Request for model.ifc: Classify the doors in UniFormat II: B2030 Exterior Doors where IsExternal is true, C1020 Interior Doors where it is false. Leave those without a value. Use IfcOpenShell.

First a look at what the model holds.

```python
import ifcopenshell
import ifcopenshell.util.element

model = ifcopenshell.open("model.ifc")
print(model.schema)
print("classifications:", [c.Name for c in model.by_type("IfcClassification")])
values = [ifcopenshell.util.element.get_pset(e, "Pset_DoorCommon", "IsExternal") for e in model.by_type("IfcDoor")]
for value in (True, False, None):
    print("IsExternal", value, values.count(value))
```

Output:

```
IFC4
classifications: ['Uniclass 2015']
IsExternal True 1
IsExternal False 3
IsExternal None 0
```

```python
import ifcopenshell
import ifcopenshell.api.classification
import ifcopenshell.util.element

model = ifcopenshell.open("model.ifc")

system = ifcopenshell.api.classification.add_classification(model, classification="UniFormat II")

doors = model.by_type("IfcDoor")
external = {e: ifcopenshell.util.element.get_pset(e, "Pset_DoorCommon", "IsExternal") for e in doors}
for flag, code, name in ((True, "B2030", "Exterior Doors"), (False, "C1020", "Interior Doors")):
    products = [e for e in doors if external[e] is flag]
    ifcopenshell.api.classification.add_reference(
        model, products=products, classification=system, identification=code, name=name
    )
    print(code, len(products))

model.write("model_updated.ifc")
```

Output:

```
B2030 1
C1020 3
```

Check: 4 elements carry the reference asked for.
